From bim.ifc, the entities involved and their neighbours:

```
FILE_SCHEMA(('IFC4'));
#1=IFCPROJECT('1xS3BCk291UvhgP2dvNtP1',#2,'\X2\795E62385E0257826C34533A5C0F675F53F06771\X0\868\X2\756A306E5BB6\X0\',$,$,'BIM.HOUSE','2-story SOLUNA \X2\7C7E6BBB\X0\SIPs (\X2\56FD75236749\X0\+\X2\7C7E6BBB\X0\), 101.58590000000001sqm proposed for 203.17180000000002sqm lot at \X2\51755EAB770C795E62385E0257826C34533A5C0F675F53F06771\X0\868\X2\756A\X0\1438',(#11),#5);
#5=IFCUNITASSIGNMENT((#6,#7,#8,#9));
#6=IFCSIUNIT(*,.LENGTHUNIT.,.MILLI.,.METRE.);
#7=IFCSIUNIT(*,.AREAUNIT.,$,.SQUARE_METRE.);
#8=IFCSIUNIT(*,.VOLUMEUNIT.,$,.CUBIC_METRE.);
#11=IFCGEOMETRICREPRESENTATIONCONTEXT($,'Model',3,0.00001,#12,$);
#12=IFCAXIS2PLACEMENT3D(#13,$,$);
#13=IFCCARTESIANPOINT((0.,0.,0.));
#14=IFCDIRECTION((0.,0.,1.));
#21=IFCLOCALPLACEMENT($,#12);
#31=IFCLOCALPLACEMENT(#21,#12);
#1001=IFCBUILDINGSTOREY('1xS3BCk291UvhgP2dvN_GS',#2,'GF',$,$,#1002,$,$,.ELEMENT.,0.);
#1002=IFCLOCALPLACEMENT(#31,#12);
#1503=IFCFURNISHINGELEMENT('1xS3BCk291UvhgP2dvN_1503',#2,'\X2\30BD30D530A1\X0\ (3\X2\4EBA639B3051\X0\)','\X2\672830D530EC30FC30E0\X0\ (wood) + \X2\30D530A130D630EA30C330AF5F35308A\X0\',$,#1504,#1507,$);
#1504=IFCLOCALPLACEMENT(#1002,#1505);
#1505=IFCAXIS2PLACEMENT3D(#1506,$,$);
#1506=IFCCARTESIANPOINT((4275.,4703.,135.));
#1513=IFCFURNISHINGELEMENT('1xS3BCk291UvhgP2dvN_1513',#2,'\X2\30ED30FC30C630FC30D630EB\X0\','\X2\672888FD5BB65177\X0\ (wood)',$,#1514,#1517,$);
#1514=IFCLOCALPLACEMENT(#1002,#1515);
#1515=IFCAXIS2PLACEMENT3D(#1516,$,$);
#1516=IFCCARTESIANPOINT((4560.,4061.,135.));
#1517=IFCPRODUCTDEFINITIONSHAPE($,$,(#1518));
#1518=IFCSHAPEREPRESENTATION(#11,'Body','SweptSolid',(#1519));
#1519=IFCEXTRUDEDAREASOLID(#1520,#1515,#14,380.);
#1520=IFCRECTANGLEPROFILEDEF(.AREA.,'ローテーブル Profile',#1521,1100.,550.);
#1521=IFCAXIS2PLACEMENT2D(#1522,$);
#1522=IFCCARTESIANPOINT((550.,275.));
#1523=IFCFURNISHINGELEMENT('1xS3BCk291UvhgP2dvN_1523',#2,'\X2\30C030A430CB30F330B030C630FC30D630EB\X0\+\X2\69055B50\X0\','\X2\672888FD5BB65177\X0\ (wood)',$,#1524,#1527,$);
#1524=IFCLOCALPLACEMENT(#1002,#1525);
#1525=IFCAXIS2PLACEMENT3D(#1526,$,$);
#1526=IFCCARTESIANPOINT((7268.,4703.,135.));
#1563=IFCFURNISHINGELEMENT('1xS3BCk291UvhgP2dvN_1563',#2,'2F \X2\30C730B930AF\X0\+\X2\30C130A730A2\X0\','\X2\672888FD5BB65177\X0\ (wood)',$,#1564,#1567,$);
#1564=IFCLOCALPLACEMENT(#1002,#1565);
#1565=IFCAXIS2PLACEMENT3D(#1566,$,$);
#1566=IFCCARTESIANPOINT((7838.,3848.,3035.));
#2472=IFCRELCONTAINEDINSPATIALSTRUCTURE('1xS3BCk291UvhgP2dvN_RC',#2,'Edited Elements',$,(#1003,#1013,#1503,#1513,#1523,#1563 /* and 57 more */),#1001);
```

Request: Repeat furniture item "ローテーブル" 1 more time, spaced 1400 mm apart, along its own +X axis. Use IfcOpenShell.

```python
import ifcopenshell
import ifcopenshell.api.geometry
import ifcopenshell.api.root
import ifcopenshell.util.element
import ifcopenshell.util.placement

model = ifcopenshell.open("bim.ifc")


def reuse_history(source, copy):
    """copy_class also copies each property set's owner history, people and application; keep the originals."""
    for rel in copy.IsDefinedBy:
        if rel.is_a("IfcRelDefinesByProperties") and (history := rel.RelatingPropertyDefinition.OwnerHistory):
            rel.RelatingPropertyDefinition.OwnerHistory = source.OwnerHistory
            ifcopenshell.util.element.remove_deep2(model, history)


source = model.by_guid("1xS3BCk291UvhgP2dvN_1513")
base = ifcopenshell.util.placement.get_local_placement(source.ObjectPlacement)
step = base[:3, 0] * 1400.0

for i in range(1, 2):
    copy = ifcopenshell.api.root.copy_class(model, product=source)
    copy.Representation = ifcopenshell.util.element.copy_deep(
        model, source.Representation, exclude=["IfcGeometricRepresentationContext", "IfcRepresentationMap"]
    )
    reuse_history(source, copy)
    matrix = base.copy()
    matrix[:3, 3] += i * step
    print("added at", matrix[:3, 3].round(3) + 0.0)
    ifcopenshell.api.geometry.edit_object_placement(model, product=copy, matrix=matrix, is_si=False)

model.write("bim_v2.ifc")
```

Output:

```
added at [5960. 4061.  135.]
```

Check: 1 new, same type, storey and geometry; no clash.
